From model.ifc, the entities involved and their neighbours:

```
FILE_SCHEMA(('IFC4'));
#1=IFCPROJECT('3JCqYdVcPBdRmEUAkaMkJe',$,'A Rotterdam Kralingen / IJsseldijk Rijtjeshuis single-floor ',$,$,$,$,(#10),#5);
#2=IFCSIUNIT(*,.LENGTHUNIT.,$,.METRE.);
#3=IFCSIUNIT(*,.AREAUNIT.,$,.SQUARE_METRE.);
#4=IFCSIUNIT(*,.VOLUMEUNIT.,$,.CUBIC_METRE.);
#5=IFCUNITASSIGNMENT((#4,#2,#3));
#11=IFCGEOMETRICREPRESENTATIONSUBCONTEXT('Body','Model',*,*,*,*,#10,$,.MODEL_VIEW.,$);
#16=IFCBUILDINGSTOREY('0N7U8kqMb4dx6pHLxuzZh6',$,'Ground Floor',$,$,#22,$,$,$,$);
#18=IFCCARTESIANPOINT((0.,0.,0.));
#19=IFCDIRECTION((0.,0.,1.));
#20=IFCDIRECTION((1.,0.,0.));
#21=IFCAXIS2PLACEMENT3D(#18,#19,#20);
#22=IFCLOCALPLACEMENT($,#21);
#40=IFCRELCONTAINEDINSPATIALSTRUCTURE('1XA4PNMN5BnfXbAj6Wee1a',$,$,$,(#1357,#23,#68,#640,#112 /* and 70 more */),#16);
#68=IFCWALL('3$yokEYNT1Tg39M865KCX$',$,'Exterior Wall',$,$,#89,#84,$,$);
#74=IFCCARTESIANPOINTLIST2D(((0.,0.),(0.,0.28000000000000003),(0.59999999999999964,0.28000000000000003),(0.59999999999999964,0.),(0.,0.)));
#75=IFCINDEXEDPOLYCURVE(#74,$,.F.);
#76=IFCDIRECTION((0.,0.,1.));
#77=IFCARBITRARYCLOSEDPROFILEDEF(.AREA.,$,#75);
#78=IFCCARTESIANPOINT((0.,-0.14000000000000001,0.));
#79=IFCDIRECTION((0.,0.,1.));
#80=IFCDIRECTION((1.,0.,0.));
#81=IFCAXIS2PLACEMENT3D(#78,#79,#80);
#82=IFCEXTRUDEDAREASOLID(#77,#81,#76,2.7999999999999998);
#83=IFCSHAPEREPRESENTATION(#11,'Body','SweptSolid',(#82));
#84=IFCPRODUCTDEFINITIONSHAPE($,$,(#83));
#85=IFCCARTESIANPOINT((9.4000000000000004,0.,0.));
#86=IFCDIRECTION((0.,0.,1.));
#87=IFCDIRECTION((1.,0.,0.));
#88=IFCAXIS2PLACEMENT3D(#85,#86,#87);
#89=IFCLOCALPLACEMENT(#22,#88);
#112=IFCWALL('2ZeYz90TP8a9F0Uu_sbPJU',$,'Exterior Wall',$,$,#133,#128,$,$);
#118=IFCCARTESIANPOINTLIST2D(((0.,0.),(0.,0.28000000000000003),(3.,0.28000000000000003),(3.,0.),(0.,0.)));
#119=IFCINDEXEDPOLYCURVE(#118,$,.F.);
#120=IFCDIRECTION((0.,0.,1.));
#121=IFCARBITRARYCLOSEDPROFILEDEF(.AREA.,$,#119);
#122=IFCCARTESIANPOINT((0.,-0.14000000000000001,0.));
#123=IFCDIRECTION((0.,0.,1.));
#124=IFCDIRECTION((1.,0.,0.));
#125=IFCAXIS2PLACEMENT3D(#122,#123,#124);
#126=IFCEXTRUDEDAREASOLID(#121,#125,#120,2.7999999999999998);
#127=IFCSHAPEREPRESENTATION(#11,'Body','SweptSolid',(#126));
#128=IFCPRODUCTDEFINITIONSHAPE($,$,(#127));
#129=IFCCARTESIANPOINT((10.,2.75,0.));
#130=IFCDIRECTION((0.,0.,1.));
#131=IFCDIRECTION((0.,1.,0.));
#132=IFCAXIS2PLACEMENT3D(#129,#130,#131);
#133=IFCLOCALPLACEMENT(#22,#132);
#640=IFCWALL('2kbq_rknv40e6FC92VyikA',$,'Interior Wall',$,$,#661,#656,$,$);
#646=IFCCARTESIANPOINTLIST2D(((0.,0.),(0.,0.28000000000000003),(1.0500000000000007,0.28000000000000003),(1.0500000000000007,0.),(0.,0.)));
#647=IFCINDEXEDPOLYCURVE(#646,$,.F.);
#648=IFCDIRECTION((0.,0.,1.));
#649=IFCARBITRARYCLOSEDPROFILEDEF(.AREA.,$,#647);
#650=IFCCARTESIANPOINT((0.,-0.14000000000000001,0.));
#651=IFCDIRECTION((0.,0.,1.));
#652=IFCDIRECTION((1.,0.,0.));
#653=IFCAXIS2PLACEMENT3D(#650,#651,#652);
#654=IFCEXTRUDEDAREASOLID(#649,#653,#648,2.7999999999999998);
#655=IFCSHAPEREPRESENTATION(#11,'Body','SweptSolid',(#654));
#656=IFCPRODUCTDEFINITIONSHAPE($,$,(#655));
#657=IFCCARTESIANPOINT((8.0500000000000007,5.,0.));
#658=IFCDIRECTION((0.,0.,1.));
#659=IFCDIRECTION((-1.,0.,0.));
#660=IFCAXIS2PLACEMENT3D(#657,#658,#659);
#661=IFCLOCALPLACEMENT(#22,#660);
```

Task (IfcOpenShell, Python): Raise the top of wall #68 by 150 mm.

```python
import ifcopenshell
import ifcopenshell.geom
import ifcopenshell.util.representation
import ifcopenshell.util.shape
import ifcopenshell.util.unit

model = ifcopenshell.open("model.ifc")
unit_scale = ifcopenshell.util.unit.calculate_unit_scale(model)
settings = ifcopenshell.geom.settings()


def volume(element):
    """Net volume in cubic metres, openings subtracted."""
    shape = ifcopenshell.geom.create_shape(settings, element)
    return ifcopenshell.util.shape.get_volume(shape.geometry)


wall = model.by_id(68)
before = volume(wall)

body = ifcopenshell.util.representation.get_representation(wall, "Model", "Body")
solid = body.Items[0]
old_height = solid.Depth
solid.Depth += 0.15 / unit_scale
after = volume(wall)

print(f"height {old_height:g} -> {solid.Depth:g}, volume {before:.3f} -> {after:.3f} m3")

model.write("model-out.ifc")
```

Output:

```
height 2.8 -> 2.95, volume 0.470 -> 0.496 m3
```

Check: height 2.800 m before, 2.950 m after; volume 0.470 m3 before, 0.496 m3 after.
